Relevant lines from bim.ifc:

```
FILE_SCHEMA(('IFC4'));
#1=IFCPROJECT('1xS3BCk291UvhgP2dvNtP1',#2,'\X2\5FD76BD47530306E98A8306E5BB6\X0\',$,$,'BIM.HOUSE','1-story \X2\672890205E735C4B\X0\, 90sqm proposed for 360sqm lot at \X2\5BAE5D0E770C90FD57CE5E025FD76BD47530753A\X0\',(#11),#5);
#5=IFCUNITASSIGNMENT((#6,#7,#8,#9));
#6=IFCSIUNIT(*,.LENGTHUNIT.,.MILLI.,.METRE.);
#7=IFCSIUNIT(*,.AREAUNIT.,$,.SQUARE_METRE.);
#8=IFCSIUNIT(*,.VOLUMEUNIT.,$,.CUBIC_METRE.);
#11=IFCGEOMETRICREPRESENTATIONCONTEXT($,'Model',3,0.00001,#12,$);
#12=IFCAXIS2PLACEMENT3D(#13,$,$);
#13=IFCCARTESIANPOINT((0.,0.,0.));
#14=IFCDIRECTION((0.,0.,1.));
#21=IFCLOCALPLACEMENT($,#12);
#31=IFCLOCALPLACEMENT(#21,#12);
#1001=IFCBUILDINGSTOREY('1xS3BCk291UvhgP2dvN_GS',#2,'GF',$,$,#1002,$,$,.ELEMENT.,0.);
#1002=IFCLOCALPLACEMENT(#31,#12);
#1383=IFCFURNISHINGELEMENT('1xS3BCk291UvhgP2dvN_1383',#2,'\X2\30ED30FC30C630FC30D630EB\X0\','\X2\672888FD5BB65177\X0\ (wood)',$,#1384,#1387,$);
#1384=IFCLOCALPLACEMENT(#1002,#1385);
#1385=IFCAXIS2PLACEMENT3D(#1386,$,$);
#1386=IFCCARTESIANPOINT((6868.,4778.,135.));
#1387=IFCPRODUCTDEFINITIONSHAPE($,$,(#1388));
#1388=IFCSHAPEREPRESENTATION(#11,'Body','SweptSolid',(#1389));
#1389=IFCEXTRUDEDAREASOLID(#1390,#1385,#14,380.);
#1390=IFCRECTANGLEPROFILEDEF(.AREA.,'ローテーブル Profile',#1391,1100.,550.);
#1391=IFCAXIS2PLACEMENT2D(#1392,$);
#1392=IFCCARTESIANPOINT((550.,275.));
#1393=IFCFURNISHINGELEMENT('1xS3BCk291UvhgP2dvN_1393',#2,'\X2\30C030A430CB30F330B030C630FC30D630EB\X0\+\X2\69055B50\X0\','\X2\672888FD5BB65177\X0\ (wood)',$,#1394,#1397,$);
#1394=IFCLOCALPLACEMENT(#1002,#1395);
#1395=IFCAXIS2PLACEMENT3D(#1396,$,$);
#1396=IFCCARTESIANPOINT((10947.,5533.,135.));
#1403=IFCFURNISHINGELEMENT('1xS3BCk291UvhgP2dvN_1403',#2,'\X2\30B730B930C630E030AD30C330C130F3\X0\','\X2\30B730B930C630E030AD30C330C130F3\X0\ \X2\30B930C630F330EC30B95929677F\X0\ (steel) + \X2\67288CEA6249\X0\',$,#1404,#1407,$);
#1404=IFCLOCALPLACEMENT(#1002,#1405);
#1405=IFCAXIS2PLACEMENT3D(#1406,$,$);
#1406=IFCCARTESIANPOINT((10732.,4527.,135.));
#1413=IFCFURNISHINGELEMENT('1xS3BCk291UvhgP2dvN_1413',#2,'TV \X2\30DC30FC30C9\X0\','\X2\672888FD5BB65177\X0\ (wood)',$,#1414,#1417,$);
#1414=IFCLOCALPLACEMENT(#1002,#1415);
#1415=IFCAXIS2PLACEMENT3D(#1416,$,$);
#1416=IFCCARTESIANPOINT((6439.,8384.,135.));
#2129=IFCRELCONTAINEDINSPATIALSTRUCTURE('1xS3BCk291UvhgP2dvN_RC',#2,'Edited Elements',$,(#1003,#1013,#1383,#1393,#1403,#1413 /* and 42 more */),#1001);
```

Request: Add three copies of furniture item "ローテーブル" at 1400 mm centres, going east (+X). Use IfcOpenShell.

```python
import numpy as np
import ifcopenshell
import ifcopenshell.api.geometry
import ifcopenshell.api.root
import ifcopenshell.util.element
import ifcopenshell.util.placement

model = ifcopenshell.open("bim.ifc")


def reuse_history(source, copy):
    """copy_class also copies each property set's owner history, people and application; keep the originals."""
    for rel in copy.IsDefinedBy:
        if rel.is_a("IfcRelDefinesByProperties") and (history := rel.RelatingPropertyDefinition.OwnerHistory):
            rel.RelatingPropertyDefinition.OwnerHistory = source.OwnerHistory
            ifcopenshell.util.element.remove_deep2(model, history)


source = model.by_guid("1xS3BCk291UvhgP2dvN_1383")
base = ifcopenshell.util.placement.get_local_placement(source.ObjectPlacement)
step = np.array([1.0, 0.0, 0.0]) * 1400.0

for i in range(1, 4):
    copy = ifcopenshell.api.root.copy_class(model, product=source)
    copy.Representation = ifcopenshell.util.element.copy_deep(
        model, source.Representation, exclude=["IfcGeometricRepresentationContext", "IfcRepresentationMap"]
    )
    reuse_history(source, copy)
    matrix = base.copy()
    matrix[:3, 3] += i * step
    print("added at", matrix[:3, 3].round(3) + 0.0)
    ifcopenshell.api.geometry.edit_object_placement(model, product=copy, matrix=matrix, is_si=False)

model.write("bim_updated.ifc")
```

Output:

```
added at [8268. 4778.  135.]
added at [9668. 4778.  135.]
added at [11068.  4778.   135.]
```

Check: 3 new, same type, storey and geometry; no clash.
